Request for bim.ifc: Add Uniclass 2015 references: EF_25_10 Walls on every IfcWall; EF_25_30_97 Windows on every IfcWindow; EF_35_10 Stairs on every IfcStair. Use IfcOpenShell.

First a look at what the model holds.

```python
import ifcopenshell

model = ifcopenshell.open("bim.ifc")
print(model.schema)
print("classifications:", [c.Name for c in model.by_type("IfcClassification")])
for ifc_class in ("IfcDoor", "IfcRoof", "IfcStair", "IfcWall", "IfcWindow"):
    print(ifc_class, len(model.by_type(ifc_class)))
```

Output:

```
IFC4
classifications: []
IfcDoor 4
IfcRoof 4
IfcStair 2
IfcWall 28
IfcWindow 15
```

```python
import ifcopenshell
import ifcopenshell.api.classification

model = ifcopenshell.open("bim.ifc")

system = ifcopenshell.api.classification.add_classification(model, classification="Uniclass 2015")

codes = {
    "IfcWall": ("EF_25_10", "Walls"),
    "IfcWindow": ("EF_25_30_97", "Windows"),
    "IfcStair": ("EF_35_10", "Stairs"),
}
for ifc_class, (code, name) in codes.items():
    products = model.by_type(ifc_class)
    ifcopenshell.api.classification.add_reference(
        model, products=products, classification=system, identification=code, name=name
    )
    print(code, len(products))

model.write("bim-out.ifc")
```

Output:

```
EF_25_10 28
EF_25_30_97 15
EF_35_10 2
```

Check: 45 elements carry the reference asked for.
